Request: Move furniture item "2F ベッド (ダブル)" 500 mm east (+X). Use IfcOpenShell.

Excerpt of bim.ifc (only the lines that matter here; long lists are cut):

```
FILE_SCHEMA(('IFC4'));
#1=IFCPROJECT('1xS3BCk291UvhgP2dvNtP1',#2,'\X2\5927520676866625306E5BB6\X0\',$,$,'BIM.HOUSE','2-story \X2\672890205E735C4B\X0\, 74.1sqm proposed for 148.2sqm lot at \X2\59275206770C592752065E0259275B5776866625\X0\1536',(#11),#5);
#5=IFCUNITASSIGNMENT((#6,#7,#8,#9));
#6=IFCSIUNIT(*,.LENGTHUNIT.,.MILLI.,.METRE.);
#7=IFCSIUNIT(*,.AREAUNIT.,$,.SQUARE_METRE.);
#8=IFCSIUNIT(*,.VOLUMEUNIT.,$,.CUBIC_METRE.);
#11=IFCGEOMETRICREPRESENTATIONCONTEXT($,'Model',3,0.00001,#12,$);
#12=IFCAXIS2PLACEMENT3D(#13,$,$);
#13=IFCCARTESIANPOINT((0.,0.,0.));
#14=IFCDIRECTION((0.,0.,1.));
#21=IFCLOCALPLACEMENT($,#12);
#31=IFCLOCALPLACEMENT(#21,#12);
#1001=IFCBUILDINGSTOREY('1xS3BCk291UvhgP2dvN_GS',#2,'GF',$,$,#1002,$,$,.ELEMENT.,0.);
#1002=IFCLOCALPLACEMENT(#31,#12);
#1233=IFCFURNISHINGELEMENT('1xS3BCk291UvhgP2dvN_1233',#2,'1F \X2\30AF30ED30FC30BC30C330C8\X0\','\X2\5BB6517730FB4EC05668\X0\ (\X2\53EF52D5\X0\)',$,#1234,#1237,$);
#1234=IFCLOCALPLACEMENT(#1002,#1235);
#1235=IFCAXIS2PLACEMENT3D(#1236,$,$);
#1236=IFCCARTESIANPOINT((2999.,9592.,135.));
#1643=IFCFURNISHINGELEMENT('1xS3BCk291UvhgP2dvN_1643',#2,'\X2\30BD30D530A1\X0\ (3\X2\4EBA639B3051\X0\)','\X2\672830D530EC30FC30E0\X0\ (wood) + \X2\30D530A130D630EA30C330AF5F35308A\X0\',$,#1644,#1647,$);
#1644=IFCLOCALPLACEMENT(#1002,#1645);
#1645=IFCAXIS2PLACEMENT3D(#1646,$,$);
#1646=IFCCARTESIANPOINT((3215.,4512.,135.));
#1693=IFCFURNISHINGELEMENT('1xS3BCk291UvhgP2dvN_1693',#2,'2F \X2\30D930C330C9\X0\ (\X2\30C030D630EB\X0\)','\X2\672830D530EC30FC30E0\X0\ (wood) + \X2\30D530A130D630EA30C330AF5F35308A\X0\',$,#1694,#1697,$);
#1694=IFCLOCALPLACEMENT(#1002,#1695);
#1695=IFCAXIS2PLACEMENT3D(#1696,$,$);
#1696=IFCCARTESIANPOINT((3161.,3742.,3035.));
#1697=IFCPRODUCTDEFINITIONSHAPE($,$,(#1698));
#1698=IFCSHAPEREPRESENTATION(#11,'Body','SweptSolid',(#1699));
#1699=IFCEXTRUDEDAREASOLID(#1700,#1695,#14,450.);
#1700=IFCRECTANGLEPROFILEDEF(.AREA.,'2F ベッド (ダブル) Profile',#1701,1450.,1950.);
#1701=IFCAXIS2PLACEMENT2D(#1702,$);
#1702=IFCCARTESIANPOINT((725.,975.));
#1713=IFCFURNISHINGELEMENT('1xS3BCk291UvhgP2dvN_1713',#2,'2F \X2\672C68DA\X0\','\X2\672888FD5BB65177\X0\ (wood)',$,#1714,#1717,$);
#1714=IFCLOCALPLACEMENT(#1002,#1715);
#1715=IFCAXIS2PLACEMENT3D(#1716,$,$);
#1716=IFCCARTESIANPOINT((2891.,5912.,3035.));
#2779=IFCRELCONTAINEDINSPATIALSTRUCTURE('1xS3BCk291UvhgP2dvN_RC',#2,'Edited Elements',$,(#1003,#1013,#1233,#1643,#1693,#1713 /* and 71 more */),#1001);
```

```python
import ifcopenshell
import ifcopenshell.api.geometry
import ifcopenshell.util.placement

model = ifcopenshell.open("bim.ifc")

item = model.by_id(1693)
matrix = ifcopenshell.util.placement.get_local_placement(item.ObjectPlacement)
matrix[0, 3] += 500.0
ifcopenshell.api.geometry.edit_object_placement(model, product=item, matrix=matrix, is_si=False)

print(ifcopenshell.util.placement.get_local_placement(item.ObjectPlacement).round(3) + 0.0)

model.write("bim_rev.ifc")
```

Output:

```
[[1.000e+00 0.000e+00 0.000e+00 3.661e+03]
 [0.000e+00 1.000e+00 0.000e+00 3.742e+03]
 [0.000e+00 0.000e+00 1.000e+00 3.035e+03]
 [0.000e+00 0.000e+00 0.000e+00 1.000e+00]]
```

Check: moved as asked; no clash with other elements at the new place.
